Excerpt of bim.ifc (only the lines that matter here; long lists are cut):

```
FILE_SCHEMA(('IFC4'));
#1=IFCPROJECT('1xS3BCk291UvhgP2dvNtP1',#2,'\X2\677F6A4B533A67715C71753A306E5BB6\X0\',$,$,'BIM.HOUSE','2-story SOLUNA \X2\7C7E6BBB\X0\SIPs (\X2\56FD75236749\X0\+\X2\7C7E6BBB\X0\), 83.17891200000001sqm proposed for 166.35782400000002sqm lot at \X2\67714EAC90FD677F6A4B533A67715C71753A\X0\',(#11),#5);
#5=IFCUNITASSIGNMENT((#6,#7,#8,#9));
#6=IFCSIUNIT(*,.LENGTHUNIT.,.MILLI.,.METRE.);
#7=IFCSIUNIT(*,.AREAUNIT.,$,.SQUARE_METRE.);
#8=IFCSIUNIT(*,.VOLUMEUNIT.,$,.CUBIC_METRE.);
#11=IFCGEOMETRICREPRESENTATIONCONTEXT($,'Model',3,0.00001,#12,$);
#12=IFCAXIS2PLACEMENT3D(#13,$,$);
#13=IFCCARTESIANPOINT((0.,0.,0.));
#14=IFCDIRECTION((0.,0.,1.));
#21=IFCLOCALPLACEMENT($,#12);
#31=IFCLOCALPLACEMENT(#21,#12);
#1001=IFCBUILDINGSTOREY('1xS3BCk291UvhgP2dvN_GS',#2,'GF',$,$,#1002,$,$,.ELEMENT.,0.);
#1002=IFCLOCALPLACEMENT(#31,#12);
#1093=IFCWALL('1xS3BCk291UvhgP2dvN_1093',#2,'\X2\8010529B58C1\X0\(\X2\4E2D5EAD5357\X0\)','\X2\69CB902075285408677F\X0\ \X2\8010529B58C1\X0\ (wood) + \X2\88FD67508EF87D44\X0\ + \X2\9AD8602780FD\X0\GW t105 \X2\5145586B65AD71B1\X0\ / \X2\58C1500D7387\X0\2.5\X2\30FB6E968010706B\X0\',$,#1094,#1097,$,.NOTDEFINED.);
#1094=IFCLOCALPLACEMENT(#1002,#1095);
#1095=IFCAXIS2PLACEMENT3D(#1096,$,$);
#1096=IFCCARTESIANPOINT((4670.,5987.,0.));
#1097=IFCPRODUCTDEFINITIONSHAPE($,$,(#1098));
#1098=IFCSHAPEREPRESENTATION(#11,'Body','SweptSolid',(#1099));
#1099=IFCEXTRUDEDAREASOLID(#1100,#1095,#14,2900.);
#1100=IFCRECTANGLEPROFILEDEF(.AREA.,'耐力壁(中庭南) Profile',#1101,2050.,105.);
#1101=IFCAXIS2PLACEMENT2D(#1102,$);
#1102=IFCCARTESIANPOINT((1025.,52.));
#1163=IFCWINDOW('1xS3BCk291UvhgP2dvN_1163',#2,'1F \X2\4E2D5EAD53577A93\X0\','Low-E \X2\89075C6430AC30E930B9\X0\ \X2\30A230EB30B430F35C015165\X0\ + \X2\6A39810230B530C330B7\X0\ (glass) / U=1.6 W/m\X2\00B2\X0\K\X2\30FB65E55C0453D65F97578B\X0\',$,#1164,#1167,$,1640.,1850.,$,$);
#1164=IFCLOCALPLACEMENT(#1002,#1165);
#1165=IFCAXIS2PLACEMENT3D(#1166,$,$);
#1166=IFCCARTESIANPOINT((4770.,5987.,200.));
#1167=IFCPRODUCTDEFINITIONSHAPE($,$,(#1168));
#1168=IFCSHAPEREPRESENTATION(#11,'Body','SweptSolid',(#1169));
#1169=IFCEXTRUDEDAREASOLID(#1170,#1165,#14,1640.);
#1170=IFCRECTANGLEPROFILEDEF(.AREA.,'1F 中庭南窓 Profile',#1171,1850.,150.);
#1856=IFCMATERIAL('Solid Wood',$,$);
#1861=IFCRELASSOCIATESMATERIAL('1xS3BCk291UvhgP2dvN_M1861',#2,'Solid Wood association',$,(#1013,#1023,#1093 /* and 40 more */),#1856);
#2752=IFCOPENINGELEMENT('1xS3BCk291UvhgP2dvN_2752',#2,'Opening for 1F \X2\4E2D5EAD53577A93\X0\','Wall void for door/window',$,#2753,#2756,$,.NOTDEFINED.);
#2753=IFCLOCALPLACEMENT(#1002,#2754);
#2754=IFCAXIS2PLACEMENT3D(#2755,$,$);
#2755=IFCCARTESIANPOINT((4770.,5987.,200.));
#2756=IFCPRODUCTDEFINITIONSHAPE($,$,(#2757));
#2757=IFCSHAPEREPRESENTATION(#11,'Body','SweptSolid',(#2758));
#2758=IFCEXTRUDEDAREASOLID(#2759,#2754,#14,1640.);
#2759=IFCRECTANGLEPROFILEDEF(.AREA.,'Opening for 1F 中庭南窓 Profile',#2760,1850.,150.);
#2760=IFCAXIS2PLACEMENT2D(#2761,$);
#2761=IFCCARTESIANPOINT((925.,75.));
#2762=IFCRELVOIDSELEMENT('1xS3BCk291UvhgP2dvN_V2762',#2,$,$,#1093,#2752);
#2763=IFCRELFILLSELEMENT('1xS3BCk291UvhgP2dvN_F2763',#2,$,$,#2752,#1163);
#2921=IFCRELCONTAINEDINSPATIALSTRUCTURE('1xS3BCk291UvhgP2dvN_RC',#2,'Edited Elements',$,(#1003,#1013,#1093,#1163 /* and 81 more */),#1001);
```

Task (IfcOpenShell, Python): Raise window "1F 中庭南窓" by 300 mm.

```python
import numpy as np
import ifcopenshell
import ifcopenshell.api.geometry
import ifcopenshell.util.placement
import ifcopenshell.util.unit

model = ifcopenshell.open("bim.ifc")
unit_scale = ifcopenshell.util.unit.calculate_unit_scale(model)

window = model.by_guid("1xS3BCk291UvhgP2dvN_1163")
opening = window.FillsVoids[0].RelatingOpeningElement
dz = 0.3 / unit_scale

shift = np.array([0.0, 0.0, dz])
# The window is not placed relative to its opening, so move both.
for product in (opening, window):
    matrix = ifcopenshell.util.placement.get_local_placement(product.ObjectPlacement)
    matrix[:3, 3] += shift
    ifcopenshell.api.geometry.edit_object_placement(model, product=product, matrix=matrix, is_si=False)

print(f"moved by {dz * unit_scale:+.3f} m")

model.write("bim_edited.ifc")
```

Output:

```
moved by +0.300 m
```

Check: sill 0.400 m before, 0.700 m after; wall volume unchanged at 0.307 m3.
